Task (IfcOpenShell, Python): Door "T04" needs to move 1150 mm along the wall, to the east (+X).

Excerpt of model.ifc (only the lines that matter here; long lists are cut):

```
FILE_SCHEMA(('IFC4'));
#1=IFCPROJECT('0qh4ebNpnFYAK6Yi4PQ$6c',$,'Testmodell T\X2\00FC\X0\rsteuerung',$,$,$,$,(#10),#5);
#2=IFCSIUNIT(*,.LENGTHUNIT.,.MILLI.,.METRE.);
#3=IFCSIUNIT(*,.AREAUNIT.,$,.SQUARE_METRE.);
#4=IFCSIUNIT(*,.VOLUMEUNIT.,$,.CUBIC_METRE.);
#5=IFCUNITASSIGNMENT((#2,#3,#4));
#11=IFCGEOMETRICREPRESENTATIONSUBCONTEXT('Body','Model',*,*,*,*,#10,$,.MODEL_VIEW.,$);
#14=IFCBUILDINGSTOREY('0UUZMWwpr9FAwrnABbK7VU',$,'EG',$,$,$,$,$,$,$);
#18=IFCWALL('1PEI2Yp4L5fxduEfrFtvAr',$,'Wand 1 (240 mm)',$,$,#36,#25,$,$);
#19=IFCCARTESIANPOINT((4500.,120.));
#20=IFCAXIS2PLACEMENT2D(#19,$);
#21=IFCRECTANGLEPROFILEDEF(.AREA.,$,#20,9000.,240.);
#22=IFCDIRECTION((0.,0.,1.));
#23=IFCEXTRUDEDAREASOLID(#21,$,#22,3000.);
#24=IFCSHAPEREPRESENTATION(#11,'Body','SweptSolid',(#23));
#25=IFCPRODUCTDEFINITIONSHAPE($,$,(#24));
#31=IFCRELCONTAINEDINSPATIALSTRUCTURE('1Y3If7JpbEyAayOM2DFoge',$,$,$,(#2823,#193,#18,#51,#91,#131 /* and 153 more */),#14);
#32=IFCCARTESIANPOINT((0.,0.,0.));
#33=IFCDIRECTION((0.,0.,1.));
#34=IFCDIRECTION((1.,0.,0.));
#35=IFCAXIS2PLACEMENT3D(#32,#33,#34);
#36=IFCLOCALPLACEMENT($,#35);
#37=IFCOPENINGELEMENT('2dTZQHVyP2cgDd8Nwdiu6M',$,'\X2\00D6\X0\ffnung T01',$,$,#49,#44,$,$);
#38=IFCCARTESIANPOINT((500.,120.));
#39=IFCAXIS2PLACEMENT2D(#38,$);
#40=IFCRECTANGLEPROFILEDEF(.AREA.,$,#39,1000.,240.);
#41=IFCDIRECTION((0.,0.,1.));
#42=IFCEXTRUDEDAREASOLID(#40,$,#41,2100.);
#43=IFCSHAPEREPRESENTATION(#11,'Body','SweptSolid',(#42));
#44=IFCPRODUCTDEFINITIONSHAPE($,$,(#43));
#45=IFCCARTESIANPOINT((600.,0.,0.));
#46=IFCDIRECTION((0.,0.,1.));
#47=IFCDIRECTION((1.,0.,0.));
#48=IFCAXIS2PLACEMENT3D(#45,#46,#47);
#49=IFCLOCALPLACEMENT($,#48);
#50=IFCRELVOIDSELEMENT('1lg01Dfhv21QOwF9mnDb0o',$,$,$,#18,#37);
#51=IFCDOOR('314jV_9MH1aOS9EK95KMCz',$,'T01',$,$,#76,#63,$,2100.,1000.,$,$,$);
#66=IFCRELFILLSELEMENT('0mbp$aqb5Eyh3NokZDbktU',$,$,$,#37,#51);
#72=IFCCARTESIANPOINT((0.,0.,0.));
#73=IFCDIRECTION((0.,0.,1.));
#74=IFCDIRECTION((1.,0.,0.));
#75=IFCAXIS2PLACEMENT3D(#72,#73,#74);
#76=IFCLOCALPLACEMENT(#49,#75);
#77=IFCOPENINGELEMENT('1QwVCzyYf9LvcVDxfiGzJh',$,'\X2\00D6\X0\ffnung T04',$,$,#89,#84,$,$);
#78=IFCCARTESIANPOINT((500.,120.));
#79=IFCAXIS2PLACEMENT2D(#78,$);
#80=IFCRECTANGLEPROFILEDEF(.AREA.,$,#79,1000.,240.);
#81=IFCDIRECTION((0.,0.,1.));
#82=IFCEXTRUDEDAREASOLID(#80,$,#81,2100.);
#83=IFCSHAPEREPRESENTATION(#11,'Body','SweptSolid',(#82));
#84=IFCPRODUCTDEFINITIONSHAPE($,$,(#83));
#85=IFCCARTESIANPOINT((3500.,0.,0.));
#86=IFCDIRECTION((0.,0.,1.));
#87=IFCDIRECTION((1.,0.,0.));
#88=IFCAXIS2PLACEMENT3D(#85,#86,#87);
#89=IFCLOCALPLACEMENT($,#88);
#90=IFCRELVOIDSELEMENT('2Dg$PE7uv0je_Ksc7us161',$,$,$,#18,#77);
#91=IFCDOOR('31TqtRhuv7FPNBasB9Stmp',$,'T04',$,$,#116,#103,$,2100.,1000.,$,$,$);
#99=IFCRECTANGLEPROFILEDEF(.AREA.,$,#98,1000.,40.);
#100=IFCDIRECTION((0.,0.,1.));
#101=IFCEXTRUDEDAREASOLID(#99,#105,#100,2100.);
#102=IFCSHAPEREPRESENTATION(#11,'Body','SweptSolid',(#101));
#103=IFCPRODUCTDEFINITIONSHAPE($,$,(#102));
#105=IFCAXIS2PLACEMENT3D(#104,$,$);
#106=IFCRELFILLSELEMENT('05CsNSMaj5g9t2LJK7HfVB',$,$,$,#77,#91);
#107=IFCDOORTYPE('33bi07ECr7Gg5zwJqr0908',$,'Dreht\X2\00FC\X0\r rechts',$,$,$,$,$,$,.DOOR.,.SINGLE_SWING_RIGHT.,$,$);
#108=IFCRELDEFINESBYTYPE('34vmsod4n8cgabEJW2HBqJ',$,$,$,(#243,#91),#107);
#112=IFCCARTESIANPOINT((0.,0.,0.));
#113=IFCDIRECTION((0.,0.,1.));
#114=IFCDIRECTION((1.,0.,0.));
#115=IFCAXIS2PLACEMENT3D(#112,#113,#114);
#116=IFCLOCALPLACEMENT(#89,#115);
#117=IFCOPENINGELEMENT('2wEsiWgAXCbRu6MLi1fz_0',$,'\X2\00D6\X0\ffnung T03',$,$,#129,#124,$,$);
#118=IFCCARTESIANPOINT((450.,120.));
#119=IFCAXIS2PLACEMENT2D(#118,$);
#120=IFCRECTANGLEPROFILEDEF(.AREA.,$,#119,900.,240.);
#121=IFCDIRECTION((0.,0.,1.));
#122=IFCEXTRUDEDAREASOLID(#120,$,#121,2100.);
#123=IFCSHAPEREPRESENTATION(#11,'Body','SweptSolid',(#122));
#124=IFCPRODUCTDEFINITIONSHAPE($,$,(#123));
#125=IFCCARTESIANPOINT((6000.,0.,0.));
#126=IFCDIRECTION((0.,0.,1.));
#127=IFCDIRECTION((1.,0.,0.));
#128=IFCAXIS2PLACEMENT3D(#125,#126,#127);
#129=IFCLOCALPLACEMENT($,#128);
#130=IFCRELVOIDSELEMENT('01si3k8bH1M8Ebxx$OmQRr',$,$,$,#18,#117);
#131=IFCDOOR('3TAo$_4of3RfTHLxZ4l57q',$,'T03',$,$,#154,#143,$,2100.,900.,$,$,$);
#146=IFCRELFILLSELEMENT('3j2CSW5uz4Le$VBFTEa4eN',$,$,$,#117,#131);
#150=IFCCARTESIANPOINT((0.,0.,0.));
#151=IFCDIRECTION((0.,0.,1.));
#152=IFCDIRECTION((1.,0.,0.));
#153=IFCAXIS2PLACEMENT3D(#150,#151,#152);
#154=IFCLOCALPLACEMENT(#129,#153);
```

```python
import ifcopenshell
import ifcopenshell.api.geometry
import ifcopenshell.util.placement
import ifcopenshell.util.unit

model = ifcopenshell.open("model.ifc")
unit_scale = ifcopenshell.util.unit.calculate_unit_scale(model)

door = model.by_guid("31TqtRhuv7FPNBasB9Stmp")
opening = door.FillsVoids[0].RelatingOpeningElement
wall = opening.VoidsElements[0].RelatingBuildingElement

wall_matrix = ifcopenshell.util.placement.get_local_placement(wall.ObjectPlacement)
shift = wall_matrix[:3, 0] * 1.15 / unit_scale
before = ifcopenshell.util.placement.get_local_placement(door.ObjectPlacement)[:3, 3].copy()

# The door is placed relative to its opening, so it follows when the opening moves.
matrix = ifcopenshell.util.placement.get_local_placement(opening.ObjectPlacement)
matrix[:3, 3] += shift
ifcopenshell.api.geometry.edit_object_placement(
    model, product=opening, matrix=matrix, is_si=False, should_transform_children=True
)

after = ifcopenshell.util.placement.get_local_placement(door.ObjectPlacement)[:3, 3]
print("door moved by", (after - before).round(3) + 0.0)

model.write("model_v2.ifc")
```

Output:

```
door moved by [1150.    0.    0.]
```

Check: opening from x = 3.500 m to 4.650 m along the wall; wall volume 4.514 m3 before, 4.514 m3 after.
